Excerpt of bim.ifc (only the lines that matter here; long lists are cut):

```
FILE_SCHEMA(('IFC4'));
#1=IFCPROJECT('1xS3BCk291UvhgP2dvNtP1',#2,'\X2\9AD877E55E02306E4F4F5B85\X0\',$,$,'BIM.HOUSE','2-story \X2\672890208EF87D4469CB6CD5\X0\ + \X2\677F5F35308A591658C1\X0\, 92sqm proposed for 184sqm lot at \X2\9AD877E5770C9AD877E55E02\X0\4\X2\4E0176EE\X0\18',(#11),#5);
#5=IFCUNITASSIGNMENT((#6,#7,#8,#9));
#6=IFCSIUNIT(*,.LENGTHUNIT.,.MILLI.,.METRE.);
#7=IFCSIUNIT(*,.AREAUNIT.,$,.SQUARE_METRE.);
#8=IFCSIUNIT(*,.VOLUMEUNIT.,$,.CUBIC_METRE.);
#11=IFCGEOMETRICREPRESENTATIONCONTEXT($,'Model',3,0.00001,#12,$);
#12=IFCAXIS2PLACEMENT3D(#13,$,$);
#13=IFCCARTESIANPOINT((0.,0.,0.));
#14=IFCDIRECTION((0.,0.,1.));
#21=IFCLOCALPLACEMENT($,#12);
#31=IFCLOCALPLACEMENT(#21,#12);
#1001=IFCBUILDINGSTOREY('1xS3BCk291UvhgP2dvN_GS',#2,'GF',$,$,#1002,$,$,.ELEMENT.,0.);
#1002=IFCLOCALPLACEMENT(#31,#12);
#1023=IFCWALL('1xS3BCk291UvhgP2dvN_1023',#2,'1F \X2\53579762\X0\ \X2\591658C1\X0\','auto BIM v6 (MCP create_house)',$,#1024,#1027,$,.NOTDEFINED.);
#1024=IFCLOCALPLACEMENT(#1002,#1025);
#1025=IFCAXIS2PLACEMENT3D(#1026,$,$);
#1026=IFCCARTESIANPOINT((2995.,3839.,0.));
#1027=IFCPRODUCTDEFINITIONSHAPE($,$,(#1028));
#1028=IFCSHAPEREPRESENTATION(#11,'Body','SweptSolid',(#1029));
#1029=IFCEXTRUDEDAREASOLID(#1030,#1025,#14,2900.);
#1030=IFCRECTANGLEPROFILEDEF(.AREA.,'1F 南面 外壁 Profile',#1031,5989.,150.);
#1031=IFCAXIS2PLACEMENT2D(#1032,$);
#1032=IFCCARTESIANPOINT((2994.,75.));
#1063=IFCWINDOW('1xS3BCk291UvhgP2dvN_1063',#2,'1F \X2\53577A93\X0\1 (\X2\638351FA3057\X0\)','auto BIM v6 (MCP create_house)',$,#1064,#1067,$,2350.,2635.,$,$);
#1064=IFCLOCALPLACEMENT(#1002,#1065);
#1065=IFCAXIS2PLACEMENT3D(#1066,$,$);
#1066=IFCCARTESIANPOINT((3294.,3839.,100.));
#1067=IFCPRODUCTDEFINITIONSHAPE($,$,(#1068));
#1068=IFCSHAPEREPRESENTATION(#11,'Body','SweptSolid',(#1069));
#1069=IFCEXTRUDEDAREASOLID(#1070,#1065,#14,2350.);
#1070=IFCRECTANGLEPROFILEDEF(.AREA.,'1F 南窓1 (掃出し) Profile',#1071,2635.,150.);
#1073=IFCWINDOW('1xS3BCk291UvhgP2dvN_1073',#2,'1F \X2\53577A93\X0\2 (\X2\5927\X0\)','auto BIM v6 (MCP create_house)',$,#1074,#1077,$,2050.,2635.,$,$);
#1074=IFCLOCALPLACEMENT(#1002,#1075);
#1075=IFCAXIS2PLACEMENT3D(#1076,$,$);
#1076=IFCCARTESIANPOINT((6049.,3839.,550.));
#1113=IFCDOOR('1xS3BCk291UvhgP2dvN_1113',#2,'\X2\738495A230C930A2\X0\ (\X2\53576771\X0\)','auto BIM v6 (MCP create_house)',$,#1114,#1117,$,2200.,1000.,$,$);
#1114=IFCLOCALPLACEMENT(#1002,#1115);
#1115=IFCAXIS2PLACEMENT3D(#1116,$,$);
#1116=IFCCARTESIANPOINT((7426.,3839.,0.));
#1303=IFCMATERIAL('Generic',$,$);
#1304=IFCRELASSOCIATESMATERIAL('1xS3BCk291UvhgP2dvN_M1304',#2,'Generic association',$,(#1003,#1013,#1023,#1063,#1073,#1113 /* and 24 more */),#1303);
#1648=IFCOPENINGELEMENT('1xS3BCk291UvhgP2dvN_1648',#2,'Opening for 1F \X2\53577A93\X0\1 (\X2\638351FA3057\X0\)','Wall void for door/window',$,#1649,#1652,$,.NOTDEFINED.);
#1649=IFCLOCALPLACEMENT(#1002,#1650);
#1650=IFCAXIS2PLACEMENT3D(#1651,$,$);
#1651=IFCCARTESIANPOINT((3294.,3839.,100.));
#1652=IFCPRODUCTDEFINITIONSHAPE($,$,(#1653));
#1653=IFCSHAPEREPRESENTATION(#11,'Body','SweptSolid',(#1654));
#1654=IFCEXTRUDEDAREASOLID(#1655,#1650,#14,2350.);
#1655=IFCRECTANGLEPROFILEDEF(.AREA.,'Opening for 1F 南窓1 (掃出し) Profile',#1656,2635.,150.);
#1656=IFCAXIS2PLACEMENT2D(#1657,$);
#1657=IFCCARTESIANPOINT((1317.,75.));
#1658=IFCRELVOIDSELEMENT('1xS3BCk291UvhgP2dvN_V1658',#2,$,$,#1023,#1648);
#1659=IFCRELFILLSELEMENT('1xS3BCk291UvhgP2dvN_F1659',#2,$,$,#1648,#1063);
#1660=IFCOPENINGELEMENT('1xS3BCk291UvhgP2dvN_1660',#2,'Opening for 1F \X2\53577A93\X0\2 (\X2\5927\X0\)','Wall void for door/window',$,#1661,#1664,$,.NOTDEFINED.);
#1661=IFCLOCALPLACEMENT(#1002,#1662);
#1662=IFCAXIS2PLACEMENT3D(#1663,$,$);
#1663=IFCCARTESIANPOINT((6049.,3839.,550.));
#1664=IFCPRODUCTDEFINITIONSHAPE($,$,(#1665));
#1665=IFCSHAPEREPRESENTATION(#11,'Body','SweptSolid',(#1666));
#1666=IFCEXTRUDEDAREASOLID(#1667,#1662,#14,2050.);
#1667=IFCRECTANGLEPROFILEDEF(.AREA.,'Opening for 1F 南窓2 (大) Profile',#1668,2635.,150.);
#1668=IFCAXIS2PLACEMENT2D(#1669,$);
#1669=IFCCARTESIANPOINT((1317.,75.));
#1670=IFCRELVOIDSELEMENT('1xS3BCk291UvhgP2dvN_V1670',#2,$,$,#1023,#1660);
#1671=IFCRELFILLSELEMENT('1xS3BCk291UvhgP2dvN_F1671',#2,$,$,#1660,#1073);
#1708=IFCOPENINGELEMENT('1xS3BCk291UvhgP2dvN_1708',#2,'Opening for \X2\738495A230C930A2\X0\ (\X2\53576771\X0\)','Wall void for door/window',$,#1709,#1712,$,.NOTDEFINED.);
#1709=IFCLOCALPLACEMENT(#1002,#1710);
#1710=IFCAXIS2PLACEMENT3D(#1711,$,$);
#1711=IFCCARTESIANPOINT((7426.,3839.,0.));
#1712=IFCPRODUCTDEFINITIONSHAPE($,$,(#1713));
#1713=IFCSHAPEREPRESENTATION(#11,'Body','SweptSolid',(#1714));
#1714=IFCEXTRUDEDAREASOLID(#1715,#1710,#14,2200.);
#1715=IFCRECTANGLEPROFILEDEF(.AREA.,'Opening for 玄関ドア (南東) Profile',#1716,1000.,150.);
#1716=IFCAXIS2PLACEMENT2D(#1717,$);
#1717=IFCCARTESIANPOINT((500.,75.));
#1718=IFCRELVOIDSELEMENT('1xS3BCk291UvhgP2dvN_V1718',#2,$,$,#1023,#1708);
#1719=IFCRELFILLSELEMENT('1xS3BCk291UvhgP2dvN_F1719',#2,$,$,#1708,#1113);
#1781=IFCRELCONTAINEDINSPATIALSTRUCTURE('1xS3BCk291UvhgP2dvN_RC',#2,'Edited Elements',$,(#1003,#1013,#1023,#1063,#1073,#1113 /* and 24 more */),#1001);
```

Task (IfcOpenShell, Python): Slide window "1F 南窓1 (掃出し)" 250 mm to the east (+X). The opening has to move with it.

```python
import ifcopenshell
import ifcopenshell.api.geometry
import ifcopenshell.util.placement

model = ifcopenshell.open("bim.ifc")

window = model.by_guid("1xS3BCk291UvhgP2dvN_1063")
opening = window.FillsVoids[0].RelatingOpeningElement
wall = opening.VoidsElements[0].RelatingBuildingElement

wall_matrix = ifcopenshell.util.placement.get_local_placement(wall.ObjectPlacement)
shift = wall_matrix[:3, 0] * 250.0
before = ifcopenshell.util.placement.get_local_placement(window.ObjectPlacement)[:3, 3].copy()

# The window is not placed relative to its opening, so move both.
for product in (opening, window):
    matrix = ifcopenshell.util.placement.get_local_placement(product.ObjectPlacement)
    matrix[:3, 3] += shift
    ifcopenshell.api.geometry.edit_object_placement(model, product=product, matrix=matrix, is_si=False)

after = ifcopenshell.util.placement.get_local_placement(window.ObjectPlacement)[:3, 3]
print("window moved by", (after - before).round(3) + 0.0)

model.write("bim_updated.ifc")
```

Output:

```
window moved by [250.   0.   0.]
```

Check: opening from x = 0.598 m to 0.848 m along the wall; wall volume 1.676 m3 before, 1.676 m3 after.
